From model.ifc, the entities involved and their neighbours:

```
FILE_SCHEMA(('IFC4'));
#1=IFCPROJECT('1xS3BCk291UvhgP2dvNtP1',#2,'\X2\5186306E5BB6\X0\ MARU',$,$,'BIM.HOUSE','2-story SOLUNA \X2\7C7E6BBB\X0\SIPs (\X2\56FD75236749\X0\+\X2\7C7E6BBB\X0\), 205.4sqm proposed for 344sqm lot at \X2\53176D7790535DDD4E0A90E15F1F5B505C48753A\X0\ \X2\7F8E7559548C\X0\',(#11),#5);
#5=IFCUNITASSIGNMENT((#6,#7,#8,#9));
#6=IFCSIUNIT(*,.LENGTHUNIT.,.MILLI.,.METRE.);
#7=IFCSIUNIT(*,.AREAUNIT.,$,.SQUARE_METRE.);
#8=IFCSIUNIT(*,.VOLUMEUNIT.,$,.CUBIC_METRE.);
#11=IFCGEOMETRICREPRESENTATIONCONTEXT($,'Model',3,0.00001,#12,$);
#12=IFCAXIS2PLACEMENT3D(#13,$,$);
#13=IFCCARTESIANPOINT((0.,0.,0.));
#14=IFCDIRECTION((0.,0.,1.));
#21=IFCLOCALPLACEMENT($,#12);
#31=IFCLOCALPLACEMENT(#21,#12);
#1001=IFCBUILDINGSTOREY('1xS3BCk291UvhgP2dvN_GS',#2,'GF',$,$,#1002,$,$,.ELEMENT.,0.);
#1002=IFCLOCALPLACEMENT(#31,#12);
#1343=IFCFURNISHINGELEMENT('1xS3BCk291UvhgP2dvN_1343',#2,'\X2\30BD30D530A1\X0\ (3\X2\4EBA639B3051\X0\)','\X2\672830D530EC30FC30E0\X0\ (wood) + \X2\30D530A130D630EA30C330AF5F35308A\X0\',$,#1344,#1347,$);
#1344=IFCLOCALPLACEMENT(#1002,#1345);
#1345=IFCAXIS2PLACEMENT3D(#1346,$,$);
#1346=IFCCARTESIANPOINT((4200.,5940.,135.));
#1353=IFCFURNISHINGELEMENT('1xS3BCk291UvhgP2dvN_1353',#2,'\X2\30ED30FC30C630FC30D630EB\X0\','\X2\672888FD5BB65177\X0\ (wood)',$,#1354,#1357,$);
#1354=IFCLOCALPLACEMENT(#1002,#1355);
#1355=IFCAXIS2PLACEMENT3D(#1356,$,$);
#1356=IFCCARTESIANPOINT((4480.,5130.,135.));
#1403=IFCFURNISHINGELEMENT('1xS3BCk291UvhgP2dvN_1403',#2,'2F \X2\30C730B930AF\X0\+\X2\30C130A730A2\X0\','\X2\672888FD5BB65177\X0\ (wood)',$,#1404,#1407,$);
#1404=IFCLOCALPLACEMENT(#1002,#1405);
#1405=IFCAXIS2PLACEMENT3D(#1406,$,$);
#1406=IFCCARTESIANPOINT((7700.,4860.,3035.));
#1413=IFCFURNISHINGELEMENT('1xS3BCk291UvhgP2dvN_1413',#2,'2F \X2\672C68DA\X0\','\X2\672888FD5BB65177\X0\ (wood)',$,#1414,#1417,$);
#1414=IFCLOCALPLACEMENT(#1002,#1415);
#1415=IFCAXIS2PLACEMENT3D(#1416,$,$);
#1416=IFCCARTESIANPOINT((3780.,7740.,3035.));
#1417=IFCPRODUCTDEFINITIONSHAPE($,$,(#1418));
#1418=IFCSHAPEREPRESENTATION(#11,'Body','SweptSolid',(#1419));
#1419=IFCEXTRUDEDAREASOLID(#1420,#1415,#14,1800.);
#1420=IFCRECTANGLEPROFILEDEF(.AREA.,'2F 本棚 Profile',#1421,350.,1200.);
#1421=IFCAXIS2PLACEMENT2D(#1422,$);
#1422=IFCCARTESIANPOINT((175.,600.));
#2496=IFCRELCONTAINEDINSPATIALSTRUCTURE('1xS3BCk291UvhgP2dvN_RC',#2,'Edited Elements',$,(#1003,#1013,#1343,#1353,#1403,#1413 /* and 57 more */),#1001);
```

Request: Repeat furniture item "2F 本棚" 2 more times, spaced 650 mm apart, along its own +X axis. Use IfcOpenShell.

```python
import ifcopenshell
import ifcopenshell.api.geometry
import ifcopenshell.api.root
import ifcopenshell.util.element
import ifcopenshell.util.placement

model = ifcopenshell.open("model.ifc")


def reuse_history(source, copy):
    """copy_class also copies each property set's owner history, people and application; keep the originals."""
    for rel in copy.IsDefinedBy:
        if rel.is_a("IfcRelDefinesByProperties") and (history := rel.RelatingPropertyDefinition.OwnerHistory):
            rel.RelatingPropertyDefinition.OwnerHistory = source.OwnerHistory
            ifcopenshell.util.element.remove_deep2(model, history)


source = model.by_id(1413)
base = ifcopenshell.util.placement.get_local_placement(source.ObjectPlacement)
step = base[:3, 0] * 650.0

for i in range(1, 3):
    copy = ifcopenshell.api.root.copy_class(model, product=source)
    copy.Representation = ifcopenshell.util.element.copy_deep(
        model, source.Representation, exclude=["IfcGeometricRepresentationContext", "IfcRepresentationMap"]
    )
    reuse_history(source, copy)
    matrix = base.copy()
    matrix[:3, 3] += i * step
    print("added at", matrix[:3, 3].round(3) + 0.0)
    ifcopenshell.api.geometry.edit_object_placement(model, product=copy, matrix=matrix, is_si=False)

model.write("model_updated.ifc")
```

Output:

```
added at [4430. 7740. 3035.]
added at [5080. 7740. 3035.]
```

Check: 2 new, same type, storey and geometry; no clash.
